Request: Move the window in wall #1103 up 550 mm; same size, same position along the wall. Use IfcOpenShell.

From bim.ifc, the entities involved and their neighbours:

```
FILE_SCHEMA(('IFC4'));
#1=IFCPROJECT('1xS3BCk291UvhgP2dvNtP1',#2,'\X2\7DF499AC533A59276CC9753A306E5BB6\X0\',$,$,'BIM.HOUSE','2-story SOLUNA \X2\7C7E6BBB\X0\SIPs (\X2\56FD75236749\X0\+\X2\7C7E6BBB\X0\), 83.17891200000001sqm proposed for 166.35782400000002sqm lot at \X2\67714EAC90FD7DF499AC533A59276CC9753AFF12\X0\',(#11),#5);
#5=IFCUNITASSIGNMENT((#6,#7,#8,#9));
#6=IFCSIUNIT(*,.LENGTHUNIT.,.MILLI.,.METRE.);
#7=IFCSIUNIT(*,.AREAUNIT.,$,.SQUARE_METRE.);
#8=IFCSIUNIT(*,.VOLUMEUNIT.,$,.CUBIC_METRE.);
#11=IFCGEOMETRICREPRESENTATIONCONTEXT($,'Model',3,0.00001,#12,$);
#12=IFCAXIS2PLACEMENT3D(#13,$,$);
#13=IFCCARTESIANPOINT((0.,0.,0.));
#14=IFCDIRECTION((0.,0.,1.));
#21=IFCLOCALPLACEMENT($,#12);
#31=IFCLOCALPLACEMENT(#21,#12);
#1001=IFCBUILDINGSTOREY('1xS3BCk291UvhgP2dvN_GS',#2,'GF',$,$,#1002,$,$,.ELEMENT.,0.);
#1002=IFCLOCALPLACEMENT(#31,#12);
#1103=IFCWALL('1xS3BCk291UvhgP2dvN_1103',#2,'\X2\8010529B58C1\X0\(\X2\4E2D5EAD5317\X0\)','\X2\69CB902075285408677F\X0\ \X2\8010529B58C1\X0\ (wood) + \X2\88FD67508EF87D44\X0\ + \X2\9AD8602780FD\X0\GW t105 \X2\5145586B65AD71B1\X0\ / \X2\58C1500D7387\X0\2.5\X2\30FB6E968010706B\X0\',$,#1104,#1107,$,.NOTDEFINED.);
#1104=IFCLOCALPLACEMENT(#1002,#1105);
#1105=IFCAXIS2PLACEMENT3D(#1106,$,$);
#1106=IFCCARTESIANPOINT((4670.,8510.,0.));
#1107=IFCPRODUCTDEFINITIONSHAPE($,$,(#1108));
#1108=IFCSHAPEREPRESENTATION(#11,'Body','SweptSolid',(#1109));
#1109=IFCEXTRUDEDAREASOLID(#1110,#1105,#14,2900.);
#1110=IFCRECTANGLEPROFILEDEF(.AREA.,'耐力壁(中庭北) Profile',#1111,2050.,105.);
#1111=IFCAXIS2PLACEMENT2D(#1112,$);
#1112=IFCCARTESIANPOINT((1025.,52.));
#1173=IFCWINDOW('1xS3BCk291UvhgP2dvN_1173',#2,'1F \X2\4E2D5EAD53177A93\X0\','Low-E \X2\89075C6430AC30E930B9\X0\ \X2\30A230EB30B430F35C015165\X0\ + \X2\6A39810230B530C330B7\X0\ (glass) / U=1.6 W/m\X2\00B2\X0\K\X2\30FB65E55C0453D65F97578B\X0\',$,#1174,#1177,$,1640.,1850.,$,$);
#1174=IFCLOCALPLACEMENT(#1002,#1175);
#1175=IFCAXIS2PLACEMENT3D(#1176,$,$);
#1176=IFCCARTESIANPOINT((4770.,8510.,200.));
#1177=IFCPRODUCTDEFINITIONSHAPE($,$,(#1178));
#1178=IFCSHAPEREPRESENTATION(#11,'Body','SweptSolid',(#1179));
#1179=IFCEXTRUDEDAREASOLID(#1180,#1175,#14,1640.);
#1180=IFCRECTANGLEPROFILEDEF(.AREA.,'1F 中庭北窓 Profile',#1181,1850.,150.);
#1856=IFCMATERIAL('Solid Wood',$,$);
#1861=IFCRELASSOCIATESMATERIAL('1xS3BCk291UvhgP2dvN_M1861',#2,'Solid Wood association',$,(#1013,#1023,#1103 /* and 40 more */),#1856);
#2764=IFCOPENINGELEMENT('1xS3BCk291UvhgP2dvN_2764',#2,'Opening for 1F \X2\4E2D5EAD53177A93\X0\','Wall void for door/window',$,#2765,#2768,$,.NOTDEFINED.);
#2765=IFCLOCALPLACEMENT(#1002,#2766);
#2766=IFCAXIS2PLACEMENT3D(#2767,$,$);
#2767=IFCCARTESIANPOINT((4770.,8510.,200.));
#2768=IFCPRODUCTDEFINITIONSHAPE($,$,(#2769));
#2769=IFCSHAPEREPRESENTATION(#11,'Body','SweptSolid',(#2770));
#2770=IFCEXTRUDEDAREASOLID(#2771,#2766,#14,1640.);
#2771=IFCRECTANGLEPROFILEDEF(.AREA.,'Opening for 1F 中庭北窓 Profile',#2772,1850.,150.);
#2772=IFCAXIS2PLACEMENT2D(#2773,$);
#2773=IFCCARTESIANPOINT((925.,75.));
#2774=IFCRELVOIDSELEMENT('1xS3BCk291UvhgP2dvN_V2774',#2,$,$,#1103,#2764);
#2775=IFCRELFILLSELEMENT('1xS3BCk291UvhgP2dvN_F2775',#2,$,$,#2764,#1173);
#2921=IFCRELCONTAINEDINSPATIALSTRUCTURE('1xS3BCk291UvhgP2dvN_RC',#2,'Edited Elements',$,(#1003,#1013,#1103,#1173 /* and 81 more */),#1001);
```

```python
import numpy as np
import ifcopenshell
import ifcopenshell.api.geometry
import ifcopenshell.util.placement
import ifcopenshell.util.unit

model = ifcopenshell.open("bim.ifc")
unit_scale = ifcopenshell.util.unit.calculate_unit_scale(model)

window = model.by_guid("1xS3BCk291UvhgP2dvN_1173")
opening = window.FillsVoids[0].RelatingOpeningElement
dz = 0.55 / unit_scale

shift = np.array([0.0, 0.0, dz])
# The window is not placed relative to its opening, so move both.
for product in (opening, window):
    matrix = ifcopenshell.util.placement.get_local_placement(product.ObjectPlacement)
    matrix[:3, 3] += shift
    ifcopenshell.api.geometry.edit_object_placement(model, product=product, matrix=matrix, is_si=False)

print(f"moved by {dz * unit_scale:+.3f} m")

model.write("bim_updated.ifc")
```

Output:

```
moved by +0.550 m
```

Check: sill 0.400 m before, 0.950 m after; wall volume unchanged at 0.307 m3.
